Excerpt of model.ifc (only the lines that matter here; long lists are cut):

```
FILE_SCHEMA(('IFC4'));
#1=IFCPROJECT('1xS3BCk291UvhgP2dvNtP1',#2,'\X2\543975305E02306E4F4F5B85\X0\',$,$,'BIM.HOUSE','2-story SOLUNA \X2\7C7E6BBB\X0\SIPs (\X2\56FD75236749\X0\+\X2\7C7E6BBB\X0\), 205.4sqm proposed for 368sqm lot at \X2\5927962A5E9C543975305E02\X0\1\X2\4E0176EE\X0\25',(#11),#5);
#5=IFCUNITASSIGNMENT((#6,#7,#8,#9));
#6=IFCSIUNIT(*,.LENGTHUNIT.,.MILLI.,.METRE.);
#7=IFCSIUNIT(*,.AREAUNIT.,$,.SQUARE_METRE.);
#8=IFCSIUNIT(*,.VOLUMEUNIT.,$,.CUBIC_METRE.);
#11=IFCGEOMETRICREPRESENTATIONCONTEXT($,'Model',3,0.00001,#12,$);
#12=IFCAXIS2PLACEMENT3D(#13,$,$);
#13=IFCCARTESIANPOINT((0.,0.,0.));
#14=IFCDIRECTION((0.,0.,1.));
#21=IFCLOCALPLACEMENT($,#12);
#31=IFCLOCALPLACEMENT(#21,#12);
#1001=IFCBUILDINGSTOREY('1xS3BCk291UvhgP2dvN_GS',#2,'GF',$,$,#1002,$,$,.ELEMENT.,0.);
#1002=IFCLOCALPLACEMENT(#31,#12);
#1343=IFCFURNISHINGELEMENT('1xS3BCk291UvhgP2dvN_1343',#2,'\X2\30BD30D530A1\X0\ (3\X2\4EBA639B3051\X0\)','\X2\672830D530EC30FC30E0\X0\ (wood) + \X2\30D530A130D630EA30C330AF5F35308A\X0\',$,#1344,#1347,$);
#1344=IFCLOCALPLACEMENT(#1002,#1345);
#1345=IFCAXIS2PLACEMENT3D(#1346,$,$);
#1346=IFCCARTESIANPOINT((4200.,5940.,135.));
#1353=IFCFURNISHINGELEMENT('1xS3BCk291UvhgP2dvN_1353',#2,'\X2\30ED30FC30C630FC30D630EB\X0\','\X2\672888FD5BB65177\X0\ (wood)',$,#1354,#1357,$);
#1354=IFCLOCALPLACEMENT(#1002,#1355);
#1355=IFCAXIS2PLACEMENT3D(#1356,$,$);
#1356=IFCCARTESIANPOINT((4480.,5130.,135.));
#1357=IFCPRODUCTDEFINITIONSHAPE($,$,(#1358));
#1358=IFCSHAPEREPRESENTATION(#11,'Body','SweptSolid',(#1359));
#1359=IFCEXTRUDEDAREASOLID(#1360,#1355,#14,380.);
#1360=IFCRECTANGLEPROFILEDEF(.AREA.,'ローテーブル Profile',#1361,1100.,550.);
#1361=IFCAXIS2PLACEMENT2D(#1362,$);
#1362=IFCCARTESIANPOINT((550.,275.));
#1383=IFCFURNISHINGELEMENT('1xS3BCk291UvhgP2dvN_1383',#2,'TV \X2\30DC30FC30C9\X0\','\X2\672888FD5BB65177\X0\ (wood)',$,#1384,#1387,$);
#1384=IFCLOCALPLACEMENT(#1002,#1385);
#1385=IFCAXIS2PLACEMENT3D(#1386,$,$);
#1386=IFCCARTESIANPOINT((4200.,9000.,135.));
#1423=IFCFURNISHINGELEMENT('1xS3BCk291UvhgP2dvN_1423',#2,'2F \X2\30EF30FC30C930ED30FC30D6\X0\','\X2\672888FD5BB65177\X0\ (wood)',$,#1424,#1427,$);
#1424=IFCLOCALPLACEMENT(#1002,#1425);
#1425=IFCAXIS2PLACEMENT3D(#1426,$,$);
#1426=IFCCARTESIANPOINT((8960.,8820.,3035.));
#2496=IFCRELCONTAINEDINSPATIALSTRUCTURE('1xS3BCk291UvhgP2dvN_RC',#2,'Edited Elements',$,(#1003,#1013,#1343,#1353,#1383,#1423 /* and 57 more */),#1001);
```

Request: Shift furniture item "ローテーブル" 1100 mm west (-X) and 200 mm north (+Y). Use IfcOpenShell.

```python
import ifcopenshell
import ifcopenshell.api.geometry
import ifcopenshell.util.placement

model = ifcopenshell.open("model.ifc")

item = model.by_id(1353)
matrix = ifcopenshell.util.placement.get_local_placement(item.ObjectPlacement)
matrix[0, 3] -= 1100.0
matrix[1, 3] += 200.0
ifcopenshell.api.geometry.edit_object_placement(model, product=item, matrix=matrix, is_si=False)

print(ifcopenshell.util.placement.get_local_placement(item.ObjectPlacement).round(3) + 0.0)

model.write("model_updated.ifc")
```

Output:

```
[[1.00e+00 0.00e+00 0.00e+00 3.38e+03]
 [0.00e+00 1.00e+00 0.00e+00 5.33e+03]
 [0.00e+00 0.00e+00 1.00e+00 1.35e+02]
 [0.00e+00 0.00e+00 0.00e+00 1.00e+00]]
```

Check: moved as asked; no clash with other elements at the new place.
